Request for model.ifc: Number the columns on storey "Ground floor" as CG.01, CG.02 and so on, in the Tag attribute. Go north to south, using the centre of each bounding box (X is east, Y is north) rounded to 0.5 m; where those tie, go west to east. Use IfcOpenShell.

First a look at what the model holds.

```python
import ifcopenshell
import ifcopenshell.util.element
import ifcopenshell.util.placement

model = ifcopenshell.open("model.ifc")
print(model.schema)
storey = next(s for s in model.by_type("IfcBuildingStorey") if s.Name == "Ground floor")
columns = [e for e in ifcopenshell.util.element.get_decomposition(storey) if e.is_a("IfcColumn")]
for e in sorted(columns, key=lambda e: e.id()):
    origin = ifcopenshell.util.placement.get_local_placement(e.ObjectPlacement)[:3, 3]
    print(e.id(), e.Tag, e.Name, origin.round(2) + 0.0, sep=" | ")
```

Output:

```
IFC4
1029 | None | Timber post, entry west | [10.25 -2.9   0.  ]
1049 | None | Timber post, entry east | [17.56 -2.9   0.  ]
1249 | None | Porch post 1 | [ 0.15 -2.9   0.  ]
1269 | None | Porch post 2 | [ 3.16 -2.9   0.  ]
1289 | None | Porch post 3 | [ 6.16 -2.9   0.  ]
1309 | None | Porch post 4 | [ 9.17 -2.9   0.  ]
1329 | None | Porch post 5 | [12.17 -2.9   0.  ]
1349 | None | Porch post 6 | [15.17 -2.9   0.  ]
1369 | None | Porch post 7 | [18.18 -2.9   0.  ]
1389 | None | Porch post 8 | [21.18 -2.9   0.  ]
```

```python
import ifcopenshell
import ifcopenshell.geom
import ifcopenshell.util.element
import ifcopenshell.util.shape

model = ifcopenshell.open("model.ifc")
settings = ifcopenshell.geom.settings()
settings.set("use-world-coords", True)


def centre(element):
    shape = ifcopenshell.geom.create_shape(settings, element)
    return ifcopenshell.util.shape.get_bbox_centroid(shape.geometry)


storey = next(s for s in model.by_type("IfcBuildingStorey") if s.Name == "Ground floor")
columns = [e for e in ifcopenshell.util.element.get_decomposition(storey) if e.is_a("IfcColumn")]

# Insertion points can sit at a corner or the storey origin, so sort by the geometry (in metres).
centres = {e: centre(e) for e in columns}
columns.sort(key=lambda e: (-round(centres[e][1] / 0.5), centres[e][0]))

for i, e in enumerate(columns, start=1):
    number = f"CG.{i:02d}"
    e.Tag = number
    print(e.id(), number)

model.write("model_updated.ifc")
```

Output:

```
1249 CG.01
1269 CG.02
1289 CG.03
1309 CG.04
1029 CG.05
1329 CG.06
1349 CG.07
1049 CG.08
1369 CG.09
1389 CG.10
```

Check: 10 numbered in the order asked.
